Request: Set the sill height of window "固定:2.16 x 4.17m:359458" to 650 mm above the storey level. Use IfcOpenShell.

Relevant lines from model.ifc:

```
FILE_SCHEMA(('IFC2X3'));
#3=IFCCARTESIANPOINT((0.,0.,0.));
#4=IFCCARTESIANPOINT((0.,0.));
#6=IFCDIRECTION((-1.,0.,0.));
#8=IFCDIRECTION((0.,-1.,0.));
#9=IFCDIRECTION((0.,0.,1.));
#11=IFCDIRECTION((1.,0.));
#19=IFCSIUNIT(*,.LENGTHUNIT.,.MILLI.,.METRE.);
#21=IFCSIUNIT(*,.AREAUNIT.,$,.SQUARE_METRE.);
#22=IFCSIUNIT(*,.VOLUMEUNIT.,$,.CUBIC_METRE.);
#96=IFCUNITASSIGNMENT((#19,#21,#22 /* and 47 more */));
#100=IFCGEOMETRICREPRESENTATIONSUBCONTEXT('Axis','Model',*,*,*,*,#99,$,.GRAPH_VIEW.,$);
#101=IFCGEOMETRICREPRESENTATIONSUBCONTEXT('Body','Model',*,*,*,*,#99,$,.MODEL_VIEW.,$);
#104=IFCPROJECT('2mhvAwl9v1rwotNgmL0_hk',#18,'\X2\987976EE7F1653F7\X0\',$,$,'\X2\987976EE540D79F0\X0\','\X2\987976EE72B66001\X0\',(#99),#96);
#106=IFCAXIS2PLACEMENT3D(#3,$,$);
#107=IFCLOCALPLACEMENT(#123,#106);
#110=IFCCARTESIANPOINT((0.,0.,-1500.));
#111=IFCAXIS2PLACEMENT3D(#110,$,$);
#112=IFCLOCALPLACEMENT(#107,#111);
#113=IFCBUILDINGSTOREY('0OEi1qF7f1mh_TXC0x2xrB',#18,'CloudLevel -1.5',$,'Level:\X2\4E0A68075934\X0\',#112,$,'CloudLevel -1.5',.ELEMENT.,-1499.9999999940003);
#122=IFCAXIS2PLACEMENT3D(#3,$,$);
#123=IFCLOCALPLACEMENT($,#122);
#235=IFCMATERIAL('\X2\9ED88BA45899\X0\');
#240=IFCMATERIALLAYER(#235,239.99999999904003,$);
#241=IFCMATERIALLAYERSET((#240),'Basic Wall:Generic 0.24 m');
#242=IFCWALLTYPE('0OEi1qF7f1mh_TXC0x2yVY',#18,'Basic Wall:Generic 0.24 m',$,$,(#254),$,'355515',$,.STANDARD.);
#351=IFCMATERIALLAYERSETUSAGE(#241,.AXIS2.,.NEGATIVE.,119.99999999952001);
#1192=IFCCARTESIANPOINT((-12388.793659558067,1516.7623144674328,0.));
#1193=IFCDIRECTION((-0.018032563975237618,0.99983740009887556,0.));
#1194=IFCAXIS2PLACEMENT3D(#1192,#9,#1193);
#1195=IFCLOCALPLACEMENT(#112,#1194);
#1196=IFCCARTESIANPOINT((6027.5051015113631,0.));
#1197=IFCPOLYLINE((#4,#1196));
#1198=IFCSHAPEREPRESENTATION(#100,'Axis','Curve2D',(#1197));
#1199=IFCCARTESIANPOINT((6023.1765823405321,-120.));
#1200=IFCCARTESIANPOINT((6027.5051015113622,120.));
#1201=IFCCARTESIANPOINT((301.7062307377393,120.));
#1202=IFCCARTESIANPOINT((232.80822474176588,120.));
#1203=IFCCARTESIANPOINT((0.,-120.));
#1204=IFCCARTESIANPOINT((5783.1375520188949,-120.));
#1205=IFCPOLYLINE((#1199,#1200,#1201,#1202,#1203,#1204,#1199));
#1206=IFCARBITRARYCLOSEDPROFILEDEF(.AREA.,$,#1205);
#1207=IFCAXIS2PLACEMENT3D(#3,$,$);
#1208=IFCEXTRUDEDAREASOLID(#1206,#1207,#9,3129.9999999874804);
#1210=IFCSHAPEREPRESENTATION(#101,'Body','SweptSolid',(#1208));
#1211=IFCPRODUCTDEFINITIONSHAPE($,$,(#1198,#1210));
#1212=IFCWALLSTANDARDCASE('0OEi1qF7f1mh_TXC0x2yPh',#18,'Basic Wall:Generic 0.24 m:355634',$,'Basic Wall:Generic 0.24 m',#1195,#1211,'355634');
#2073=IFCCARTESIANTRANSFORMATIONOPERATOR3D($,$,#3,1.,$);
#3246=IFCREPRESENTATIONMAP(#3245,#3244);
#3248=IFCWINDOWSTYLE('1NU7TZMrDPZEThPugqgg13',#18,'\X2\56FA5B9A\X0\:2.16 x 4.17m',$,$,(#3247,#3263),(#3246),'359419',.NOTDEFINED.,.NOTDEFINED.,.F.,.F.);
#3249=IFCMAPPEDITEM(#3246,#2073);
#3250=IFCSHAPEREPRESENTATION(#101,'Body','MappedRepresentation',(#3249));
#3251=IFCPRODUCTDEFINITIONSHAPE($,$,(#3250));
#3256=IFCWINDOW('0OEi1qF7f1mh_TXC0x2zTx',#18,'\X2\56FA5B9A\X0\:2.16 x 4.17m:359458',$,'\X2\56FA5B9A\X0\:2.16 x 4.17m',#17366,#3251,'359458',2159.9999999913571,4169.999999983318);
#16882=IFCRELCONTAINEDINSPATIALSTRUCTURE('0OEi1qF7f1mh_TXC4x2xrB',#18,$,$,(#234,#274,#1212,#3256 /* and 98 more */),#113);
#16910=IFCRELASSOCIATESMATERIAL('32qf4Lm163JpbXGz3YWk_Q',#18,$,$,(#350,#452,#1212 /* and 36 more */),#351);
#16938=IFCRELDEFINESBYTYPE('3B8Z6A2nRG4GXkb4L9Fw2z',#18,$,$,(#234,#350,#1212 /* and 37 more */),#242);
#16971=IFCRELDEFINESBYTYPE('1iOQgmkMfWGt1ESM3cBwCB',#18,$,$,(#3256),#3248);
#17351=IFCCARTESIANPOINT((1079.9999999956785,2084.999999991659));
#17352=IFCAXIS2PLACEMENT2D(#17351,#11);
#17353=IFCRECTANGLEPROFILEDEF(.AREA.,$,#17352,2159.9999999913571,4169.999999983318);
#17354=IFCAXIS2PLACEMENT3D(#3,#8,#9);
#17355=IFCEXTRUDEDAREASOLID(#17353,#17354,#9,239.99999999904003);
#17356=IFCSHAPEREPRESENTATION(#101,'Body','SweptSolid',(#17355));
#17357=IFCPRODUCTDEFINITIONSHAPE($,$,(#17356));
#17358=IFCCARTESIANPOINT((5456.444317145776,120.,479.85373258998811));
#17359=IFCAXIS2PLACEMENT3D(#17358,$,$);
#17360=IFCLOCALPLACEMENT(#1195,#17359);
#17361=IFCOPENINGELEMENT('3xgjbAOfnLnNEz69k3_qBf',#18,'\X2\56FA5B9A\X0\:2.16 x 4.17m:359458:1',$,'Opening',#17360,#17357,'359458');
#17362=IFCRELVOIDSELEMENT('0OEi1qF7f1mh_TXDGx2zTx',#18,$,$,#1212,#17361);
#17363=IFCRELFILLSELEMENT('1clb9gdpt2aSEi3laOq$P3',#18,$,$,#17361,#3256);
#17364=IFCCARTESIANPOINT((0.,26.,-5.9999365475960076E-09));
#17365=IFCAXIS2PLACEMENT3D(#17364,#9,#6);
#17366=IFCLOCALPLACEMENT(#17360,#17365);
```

```python
import numpy as np
import ifcopenshell
import ifcopenshell.api.geometry
import ifcopenshell.geom
import ifcopenshell.util.element
import ifcopenshell.util.placement
import ifcopenshell.util.shape
import ifcopenshell.util.unit

model = ifcopenshell.open("model.ifc")
unit_scale = ifcopenshell.util.unit.calculate_unit_scale(model)

window = model.by_id(3256)
opening = window.FillsVoids[0].RelatingOpeningElement
storey = ifcopenshell.util.element.get_container(window, ifc_class="IfcBuildingStorey")
level = ifcopenshell.util.placement.get_local_placement(storey.ObjectPlacement)[2, 3]

# The opening's origin need not be at the sill, so measure its lowest point.
shape = ifcopenshell.geom.create_shape(ifcopenshell.geom.settings(), opening)
bottom = ifcopenshell.util.shape.get_shape_bottom_elevation(shape, shape.geometry) / unit_scale
dz = level + 0.65 / unit_scale - bottom

shift = np.array([0.0, 0.0, dz])
# The window is placed relative to its opening, so it follows when the opening moves.
matrix = ifcopenshell.util.placement.get_local_placement(opening.ObjectPlacement)
matrix[:3, 3] += shift
ifcopenshell.api.geometry.edit_object_placement(
    model, product=opening, matrix=matrix, is_si=False, should_transform_children=True
)

print(f"moved by {dz * unit_scale:+.3f} m")

model.write("model_edited.ifc")
```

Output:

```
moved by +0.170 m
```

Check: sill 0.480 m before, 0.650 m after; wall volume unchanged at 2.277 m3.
